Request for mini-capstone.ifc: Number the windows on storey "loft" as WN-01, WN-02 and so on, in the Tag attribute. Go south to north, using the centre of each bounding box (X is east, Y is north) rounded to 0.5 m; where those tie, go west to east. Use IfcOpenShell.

First a look at what the model holds.

```python
import ifcopenshell
import ifcopenshell.util.element
import ifcopenshell.util.placement

model = ifcopenshell.open("mini-capstone.ifc")
print(model.schema)
storey = next(s for s in model.by_type("IfcBuildingStorey") if s.Name == "loft")
windows = [e for e in ifcopenshell.util.element.get_decomposition(storey) if e.is_a("IfcWindow")]
for e in sorted(windows, key=lambda e: e.id()):
    origin = ifcopenshell.util.placement.get_local_placement(e.ObjectPlacement)[:3, 3]
    print(e.id(), e.Tag, e.Name, origin.round(2) + 0.0, sep=" | ")
```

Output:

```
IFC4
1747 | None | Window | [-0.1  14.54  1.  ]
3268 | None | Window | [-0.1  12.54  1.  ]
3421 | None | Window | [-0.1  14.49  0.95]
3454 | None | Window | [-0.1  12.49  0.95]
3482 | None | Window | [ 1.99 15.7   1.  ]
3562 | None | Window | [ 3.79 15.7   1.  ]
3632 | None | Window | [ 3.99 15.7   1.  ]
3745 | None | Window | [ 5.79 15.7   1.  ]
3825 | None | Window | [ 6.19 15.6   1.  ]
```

```python
import ifcopenshell
import ifcopenshell.geom
import ifcopenshell.util.element
import ifcopenshell.util.shape

model = ifcopenshell.open("mini-capstone.ifc")
settings = ifcopenshell.geom.settings()
settings.set("use-world-coords", True)


def centre(element):
    shape = ifcopenshell.geom.create_shape(settings, element)
    return ifcopenshell.util.shape.get_bbox_centroid(shape.geometry)


storey = next(s for s in model.by_type("IfcBuildingStorey") if s.Name == "loft")
windows = [e for e in ifcopenshell.util.element.get_decomposition(storey) if e.is_a("IfcWindow")]

# Insertion points can sit at a corner or the storey origin, so sort by the geometry (in metres).
centres = {e: centre(e) for e in windows}
windows.sort(key=lambda e: (round(centres[e][1] / 0.5), centres[e][0]))

for i, e in enumerate(windows, start=1):
    number = f"WN-{i:02d}"
    e.Tag = number
    print(e.id(), number)

model.write("mini-capstone_v2.ifc")
```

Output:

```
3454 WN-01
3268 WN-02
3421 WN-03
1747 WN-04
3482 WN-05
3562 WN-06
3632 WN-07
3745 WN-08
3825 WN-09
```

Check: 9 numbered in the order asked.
